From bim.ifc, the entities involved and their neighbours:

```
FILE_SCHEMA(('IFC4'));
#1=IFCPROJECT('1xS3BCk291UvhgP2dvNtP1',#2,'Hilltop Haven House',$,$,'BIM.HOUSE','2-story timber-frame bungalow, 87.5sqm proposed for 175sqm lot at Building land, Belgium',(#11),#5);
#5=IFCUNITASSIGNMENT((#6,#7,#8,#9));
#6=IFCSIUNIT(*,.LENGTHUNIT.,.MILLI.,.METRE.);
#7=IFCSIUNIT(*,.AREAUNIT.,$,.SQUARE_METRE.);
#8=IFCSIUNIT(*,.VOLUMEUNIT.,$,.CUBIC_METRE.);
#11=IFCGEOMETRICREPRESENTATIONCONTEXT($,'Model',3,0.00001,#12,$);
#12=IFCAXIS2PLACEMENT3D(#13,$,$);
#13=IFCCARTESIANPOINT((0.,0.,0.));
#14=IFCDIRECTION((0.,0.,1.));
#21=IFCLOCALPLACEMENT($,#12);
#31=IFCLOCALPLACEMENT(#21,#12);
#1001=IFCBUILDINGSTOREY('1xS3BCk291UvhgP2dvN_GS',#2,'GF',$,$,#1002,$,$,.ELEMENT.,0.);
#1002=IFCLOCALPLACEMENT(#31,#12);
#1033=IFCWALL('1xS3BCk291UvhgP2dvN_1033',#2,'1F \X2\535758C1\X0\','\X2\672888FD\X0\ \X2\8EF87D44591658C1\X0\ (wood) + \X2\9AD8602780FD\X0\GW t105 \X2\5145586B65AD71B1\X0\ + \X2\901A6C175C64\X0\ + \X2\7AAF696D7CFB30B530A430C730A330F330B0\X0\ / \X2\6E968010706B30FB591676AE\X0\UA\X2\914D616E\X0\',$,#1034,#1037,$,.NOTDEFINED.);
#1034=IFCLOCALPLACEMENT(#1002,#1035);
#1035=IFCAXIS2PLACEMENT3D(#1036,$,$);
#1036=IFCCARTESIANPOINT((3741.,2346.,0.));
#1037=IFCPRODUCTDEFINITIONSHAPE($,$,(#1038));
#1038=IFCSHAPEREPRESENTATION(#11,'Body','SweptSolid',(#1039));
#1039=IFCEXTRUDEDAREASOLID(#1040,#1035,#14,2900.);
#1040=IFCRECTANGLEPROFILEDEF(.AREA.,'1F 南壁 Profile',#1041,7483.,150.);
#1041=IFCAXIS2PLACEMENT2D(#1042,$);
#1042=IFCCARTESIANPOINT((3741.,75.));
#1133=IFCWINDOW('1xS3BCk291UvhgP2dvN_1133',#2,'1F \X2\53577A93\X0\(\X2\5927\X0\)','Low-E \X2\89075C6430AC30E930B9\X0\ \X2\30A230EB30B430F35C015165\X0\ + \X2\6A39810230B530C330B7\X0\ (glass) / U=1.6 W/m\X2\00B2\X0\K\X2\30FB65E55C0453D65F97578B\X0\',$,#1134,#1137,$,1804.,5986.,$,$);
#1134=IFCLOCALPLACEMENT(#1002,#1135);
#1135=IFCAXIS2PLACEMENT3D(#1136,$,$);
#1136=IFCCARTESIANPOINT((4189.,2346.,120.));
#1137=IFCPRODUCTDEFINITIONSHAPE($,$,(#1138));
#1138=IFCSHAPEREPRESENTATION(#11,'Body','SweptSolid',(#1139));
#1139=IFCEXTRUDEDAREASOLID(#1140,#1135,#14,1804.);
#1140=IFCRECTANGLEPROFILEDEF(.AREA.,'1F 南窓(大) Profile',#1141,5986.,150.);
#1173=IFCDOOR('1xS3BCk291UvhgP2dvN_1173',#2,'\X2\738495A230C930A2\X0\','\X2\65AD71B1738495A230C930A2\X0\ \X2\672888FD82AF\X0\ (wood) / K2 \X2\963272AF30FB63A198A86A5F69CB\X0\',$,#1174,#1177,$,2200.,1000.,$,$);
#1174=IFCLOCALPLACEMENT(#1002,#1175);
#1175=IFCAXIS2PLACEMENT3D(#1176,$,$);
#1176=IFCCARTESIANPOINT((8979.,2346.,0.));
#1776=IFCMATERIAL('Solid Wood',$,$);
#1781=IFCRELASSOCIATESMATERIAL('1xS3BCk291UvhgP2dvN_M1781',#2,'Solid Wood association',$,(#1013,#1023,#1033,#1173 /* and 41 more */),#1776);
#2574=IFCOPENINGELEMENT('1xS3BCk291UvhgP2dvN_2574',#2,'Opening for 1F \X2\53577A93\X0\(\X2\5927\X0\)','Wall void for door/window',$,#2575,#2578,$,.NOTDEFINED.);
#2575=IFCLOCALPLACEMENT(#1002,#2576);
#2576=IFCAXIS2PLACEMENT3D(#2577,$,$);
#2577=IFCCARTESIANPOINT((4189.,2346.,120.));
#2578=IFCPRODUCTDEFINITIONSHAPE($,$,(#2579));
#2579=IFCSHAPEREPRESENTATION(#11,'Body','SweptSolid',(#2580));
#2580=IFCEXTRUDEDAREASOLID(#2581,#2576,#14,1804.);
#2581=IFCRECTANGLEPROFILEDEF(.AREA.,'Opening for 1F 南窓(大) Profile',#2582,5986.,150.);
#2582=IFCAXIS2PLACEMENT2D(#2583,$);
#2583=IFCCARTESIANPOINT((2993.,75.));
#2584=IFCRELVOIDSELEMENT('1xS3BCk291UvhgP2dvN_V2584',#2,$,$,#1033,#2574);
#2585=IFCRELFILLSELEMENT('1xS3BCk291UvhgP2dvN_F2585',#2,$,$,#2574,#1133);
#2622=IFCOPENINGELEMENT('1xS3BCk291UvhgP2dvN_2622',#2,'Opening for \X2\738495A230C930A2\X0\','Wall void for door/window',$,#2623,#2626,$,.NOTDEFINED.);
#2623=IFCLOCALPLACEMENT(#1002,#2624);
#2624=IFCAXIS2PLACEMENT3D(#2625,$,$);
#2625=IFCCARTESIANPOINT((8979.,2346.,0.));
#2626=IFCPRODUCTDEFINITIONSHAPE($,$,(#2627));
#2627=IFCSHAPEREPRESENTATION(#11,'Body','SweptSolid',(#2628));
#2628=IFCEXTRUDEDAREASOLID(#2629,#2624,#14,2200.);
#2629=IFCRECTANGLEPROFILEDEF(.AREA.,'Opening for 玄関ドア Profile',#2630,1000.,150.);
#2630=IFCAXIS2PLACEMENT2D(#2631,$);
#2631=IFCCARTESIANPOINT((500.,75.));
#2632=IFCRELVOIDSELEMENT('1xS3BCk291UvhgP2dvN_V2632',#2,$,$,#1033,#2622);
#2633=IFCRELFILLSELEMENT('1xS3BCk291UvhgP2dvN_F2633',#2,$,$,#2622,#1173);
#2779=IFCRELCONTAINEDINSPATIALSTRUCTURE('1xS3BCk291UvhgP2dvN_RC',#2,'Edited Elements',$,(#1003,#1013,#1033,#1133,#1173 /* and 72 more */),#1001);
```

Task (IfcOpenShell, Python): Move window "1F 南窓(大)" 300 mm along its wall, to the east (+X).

```python
import ifcopenshell
import ifcopenshell.api.geometry
import ifcopenshell.util.placement

model = ifcopenshell.open("bim.ifc")

window = model.by_id(1133)
opening = window.FillsVoids[0].RelatingOpeningElement
wall = opening.VoidsElements[0].RelatingBuildingElement

wall_matrix = ifcopenshell.util.placement.get_local_placement(wall.ObjectPlacement)
shift = wall_matrix[:3, 0] * 300.0
before = ifcopenshell.util.placement.get_local_placement(window.ObjectPlacement)[:3, 3].copy()

# The window is not placed relative to its opening, so move both.
for product in (opening, window):
    matrix = ifcopenshell.util.placement.get_local_placement(product.ObjectPlacement)
    matrix[:3, 3] += shift
    ifcopenshell.api.geometry.edit_object_placement(model, product=product, matrix=matrix, is_si=False)

after = ifcopenshell.util.placement.get_local_placement(window.ObjectPlacement)[:3, 3]
print("window moved by", (after - before).round(3) + 0.0)

model.write("bim-out.ifc")
```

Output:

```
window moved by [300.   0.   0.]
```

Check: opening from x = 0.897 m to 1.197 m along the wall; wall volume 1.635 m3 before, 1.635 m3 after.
